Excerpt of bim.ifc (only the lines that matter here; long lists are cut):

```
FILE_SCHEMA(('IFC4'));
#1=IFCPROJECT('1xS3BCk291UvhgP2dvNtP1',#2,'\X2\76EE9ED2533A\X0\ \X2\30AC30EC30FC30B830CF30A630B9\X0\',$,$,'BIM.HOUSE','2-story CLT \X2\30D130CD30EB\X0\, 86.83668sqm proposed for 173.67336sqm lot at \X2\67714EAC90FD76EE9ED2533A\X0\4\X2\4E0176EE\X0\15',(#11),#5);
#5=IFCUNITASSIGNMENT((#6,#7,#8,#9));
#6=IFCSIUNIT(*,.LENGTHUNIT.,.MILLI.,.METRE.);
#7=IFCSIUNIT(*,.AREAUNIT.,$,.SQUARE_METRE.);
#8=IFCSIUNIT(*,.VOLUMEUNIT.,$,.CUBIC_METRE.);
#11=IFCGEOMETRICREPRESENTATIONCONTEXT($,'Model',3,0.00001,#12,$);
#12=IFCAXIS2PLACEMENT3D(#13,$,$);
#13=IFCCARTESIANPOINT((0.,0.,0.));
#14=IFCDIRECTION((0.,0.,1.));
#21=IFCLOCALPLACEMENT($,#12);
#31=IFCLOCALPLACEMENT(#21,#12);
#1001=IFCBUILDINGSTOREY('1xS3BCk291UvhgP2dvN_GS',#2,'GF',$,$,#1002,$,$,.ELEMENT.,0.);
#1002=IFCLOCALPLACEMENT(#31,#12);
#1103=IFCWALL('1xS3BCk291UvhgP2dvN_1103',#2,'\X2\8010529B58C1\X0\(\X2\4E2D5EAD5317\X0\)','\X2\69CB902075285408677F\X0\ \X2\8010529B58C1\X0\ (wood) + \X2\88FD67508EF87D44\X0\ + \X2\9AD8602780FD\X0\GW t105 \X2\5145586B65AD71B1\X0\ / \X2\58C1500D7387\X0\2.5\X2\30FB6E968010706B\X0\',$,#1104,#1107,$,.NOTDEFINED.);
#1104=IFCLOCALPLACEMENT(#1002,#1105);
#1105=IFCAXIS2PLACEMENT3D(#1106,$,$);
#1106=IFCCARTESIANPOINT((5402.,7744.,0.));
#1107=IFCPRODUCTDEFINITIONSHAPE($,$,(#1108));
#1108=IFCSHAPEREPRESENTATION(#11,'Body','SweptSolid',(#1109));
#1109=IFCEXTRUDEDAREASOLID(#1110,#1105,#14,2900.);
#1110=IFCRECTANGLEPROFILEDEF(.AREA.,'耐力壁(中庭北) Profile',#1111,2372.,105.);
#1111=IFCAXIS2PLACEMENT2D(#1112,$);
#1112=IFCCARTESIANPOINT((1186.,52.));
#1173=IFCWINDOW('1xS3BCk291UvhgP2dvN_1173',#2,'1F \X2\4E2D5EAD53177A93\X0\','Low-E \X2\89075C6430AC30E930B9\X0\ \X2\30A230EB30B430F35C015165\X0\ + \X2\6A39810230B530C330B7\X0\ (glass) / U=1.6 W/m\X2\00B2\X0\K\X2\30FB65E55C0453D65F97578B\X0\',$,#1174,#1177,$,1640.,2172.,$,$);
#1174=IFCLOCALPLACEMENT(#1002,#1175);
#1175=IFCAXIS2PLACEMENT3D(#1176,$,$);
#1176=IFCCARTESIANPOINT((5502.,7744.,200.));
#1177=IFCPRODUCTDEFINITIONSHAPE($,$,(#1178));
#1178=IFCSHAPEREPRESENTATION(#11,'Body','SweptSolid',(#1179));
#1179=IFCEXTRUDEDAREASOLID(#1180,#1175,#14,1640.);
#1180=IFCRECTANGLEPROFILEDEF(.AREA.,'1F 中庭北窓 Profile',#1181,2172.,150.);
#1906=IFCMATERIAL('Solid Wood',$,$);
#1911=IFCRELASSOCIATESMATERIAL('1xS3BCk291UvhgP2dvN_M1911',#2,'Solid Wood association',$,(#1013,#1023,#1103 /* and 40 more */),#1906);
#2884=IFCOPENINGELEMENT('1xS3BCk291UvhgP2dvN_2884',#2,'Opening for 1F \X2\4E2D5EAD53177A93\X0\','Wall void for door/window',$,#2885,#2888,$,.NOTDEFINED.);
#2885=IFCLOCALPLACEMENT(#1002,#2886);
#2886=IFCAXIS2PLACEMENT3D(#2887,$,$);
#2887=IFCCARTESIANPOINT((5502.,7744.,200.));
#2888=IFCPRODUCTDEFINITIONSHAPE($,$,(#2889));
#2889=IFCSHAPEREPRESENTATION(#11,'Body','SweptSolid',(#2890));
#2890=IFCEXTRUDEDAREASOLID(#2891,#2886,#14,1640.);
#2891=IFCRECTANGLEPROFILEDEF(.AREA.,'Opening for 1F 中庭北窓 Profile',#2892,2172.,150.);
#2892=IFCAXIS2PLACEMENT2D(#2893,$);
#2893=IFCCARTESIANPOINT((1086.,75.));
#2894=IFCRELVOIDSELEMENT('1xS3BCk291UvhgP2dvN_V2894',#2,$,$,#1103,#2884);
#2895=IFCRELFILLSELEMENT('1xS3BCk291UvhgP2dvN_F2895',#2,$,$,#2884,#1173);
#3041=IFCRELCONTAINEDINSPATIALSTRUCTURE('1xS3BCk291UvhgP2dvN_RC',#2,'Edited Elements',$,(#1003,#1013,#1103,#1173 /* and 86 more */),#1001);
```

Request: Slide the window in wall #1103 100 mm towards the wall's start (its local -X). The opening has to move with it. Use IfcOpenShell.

```python
import ifcopenshell
import ifcopenshell.api.geometry
import ifcopenshell.util.placement

model = ifcopenshell.open("bim.ifc")

window = model.by_id(1173)
opening = window.FillsVoids[0].RelatingOpeningElement
wall = opening.VoidsElements[0].RelatingBuildingElement

wall_matrix = ifcopenshell.util.placement.get_local_placement(wall.ObjectPlacement)
shift = wall_matrix[:3, 0] * -100.0
before = ifcopenshell.util.placement.get_local_placement(window.ObjectPlacement)[:3, 3].copy()

# The window is not placed relative to its opening, so move both.
for product in (opening, window):
    matrix = ifcopenshell.util.placement.get_local_placement(product.ObjectPlacement)
    matrix[:3, 3] += shift
    ifcopenshell.api.geometry.edit_object_placement(model, product=product, matrix=matrix, is_si=False)

after = ifcopenshell.util.placement.get_local_placement(window.ObjectPlacement)[:3, 3]
print("window moved by", (after - before).round(3) + 0.0)

model.write("bim_v2.ifc")
```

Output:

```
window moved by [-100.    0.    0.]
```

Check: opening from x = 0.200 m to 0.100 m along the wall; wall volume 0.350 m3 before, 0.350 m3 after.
